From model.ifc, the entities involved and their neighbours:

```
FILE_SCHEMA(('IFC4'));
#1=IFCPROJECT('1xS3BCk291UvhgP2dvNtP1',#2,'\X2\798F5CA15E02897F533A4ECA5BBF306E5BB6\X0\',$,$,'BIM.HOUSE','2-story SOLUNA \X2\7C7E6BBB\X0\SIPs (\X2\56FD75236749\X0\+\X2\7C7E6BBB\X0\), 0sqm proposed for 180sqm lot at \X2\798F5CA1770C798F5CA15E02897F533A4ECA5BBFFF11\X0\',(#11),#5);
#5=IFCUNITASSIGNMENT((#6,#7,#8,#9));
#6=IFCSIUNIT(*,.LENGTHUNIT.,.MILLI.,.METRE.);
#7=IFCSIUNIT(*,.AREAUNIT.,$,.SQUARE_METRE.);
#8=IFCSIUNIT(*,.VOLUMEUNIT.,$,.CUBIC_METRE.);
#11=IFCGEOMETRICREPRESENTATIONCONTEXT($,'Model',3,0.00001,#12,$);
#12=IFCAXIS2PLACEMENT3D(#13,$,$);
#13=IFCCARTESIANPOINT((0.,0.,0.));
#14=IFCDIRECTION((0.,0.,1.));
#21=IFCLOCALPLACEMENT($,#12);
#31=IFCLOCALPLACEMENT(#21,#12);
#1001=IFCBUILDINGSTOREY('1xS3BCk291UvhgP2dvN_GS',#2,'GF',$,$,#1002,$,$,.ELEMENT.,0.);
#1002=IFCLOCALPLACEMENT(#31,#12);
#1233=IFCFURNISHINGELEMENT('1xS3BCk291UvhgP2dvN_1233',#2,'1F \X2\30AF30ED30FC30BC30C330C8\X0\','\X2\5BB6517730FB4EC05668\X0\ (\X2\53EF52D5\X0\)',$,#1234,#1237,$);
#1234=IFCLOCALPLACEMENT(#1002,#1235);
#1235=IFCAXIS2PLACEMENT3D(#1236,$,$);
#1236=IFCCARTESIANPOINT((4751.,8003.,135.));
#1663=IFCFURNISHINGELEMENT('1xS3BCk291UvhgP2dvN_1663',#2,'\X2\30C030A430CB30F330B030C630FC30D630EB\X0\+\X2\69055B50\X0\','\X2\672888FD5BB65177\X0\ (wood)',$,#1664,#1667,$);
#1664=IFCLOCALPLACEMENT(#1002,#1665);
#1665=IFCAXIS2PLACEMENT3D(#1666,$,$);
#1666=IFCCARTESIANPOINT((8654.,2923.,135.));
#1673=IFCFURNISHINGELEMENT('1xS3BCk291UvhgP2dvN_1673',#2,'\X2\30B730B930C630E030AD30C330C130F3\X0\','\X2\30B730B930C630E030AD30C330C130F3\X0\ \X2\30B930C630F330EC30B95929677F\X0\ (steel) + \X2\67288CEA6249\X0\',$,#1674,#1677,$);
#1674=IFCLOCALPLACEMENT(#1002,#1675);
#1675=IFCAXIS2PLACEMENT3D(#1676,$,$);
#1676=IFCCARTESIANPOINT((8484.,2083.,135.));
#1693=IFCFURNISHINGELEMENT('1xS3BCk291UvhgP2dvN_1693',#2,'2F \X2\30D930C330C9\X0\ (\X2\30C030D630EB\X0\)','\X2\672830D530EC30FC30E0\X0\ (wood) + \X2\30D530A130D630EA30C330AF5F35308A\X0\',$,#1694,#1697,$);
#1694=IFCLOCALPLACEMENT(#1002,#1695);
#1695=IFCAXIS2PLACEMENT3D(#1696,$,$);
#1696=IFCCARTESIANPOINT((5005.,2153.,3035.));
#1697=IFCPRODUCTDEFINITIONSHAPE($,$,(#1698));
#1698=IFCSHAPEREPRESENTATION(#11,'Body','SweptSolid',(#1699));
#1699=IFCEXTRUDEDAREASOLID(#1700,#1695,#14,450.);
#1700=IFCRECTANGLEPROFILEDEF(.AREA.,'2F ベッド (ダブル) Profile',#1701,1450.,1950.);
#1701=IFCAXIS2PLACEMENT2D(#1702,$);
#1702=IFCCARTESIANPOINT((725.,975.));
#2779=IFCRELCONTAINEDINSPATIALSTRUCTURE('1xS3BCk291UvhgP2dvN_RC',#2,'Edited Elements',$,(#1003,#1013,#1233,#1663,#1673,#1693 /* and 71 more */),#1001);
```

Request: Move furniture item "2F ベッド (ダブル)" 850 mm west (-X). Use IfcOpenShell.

```python
import ifcopenshell
import ifcopenshell.api.geometry
import ifcopenshell.util.placement
import ifcopenshell.util.unit

model = ifcopenshell.open("model.ifc")
unit_scale = ifcopenshell.util.unit.calculate_unit_scale(model)

item = model.by_guid("1xS3BCk291UvhgP2dvN_1693")
matrix = ifcopenshell.util.placement.get_local_placement(item.ObjectPlacement)
matrix[0, 3] -= 0.85 / unit_scale
ifcopenshell.api.geometry.edit_object_placement(model, product=item, matrix=matrix, is_si=False)

print(ifcopenshell.util.placement.get_local_placement(item.ObjectPlacement).round(3) + 0.0)

model.write("model_v2.ifc")
```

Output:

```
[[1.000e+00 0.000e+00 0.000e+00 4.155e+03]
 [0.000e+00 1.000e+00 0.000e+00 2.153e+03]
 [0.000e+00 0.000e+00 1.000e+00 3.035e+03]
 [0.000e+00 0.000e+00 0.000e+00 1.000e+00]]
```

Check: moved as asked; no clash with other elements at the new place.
